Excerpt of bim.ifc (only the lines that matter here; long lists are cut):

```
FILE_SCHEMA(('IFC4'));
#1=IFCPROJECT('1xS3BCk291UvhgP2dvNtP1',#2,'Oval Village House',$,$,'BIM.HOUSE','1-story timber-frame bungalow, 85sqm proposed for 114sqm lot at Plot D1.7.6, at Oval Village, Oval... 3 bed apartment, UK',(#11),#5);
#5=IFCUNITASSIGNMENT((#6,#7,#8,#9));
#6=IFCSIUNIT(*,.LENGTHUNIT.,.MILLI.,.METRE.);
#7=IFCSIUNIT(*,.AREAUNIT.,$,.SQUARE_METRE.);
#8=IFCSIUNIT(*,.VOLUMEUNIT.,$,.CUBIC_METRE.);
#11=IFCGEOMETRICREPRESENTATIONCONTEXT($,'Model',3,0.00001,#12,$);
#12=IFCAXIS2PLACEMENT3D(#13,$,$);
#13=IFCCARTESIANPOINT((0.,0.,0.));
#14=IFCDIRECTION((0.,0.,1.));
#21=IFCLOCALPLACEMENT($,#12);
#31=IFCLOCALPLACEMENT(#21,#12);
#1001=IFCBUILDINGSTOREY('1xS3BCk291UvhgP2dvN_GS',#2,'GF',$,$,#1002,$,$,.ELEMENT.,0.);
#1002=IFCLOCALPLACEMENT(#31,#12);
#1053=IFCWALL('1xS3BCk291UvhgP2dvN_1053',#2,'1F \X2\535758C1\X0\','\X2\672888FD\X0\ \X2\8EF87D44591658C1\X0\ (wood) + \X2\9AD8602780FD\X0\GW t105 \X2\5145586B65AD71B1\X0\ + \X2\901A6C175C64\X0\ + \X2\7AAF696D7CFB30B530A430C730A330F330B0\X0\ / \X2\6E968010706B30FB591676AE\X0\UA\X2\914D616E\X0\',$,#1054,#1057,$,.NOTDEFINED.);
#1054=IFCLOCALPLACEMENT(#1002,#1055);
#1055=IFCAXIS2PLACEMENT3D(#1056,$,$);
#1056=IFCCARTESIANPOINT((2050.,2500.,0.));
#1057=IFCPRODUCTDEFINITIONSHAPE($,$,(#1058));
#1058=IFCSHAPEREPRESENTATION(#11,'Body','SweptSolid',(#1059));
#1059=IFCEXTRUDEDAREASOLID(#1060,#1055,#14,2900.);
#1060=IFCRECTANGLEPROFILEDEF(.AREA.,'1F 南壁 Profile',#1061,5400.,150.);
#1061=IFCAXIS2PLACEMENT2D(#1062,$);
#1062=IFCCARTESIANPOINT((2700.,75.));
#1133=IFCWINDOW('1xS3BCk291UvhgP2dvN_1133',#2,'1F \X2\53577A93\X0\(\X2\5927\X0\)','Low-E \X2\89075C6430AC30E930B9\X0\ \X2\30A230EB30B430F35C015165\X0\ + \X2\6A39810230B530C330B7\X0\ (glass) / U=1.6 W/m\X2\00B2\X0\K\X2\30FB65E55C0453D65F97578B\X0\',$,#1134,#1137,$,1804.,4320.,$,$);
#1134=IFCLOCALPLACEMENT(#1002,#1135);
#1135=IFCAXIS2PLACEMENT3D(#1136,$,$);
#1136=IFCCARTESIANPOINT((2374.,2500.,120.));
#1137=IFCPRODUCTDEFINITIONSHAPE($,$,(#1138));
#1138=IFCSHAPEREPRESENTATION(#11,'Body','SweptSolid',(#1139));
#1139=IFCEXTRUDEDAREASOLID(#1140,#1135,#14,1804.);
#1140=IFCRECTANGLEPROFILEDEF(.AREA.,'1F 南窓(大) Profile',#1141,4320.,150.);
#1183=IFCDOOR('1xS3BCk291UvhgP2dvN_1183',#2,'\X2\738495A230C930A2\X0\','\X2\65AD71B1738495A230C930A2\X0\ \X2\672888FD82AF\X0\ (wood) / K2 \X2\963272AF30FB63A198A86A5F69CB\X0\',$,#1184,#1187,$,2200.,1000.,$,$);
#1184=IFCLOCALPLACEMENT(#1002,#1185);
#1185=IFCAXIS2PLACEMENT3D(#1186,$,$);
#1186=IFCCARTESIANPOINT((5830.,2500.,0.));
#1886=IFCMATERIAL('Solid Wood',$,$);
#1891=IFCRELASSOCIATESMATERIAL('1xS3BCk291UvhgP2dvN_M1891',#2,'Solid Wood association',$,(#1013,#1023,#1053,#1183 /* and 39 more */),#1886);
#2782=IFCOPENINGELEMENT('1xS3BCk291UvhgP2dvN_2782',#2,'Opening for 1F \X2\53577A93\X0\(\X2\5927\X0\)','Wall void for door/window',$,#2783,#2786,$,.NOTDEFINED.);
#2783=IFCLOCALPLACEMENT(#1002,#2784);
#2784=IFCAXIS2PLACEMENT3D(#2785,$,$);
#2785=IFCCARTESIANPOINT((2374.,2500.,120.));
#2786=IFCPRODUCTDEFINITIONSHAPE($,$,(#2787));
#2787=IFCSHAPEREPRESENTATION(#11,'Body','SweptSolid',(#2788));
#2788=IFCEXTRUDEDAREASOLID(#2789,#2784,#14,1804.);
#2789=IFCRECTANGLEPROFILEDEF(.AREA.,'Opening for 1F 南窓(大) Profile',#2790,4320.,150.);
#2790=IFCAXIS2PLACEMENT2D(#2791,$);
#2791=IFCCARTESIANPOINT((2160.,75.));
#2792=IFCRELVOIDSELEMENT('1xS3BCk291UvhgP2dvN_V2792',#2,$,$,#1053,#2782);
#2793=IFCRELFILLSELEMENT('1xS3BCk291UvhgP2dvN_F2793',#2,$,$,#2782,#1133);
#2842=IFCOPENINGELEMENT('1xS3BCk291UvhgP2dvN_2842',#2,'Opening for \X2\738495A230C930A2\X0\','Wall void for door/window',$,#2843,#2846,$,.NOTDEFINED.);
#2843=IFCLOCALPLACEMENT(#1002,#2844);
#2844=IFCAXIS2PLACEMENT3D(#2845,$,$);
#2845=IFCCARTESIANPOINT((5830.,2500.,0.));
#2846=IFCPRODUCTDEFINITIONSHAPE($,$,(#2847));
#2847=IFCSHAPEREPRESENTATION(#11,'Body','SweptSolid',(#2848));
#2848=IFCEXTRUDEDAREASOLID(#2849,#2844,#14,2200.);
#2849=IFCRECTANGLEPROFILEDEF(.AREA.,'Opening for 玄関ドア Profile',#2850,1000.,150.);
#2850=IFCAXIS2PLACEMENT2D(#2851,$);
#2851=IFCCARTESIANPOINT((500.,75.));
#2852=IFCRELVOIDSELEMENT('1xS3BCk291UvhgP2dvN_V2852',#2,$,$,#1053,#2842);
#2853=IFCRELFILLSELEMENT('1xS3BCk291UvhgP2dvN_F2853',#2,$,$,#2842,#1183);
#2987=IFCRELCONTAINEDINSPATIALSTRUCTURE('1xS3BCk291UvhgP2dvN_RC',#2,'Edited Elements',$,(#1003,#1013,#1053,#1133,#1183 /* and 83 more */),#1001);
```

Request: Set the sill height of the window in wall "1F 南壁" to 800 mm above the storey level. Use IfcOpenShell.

```python
import numpy as np
import ifcopenshell
import ifcopenshell.api.geometry
import ifcopenshell.geom
import ifcopenshell.util.element
import ifcopenshell.util.placement
import ifcopenshell.util.shape
import ifcopenshell.util.unit

model = ifcopenshell.open("bim.ifc")
unit_scale = ifcopenshell.util.unit.calculate_unit_scale(model)

window = model.by_guid("1xS3BCk291UvhgP2dvN_1133")
opening = window.FillsVoids[0].RelatingOpeningElement
storey = ifcopenshell.util.element.get_container(window, ifc_class="IfcBuildingStorey")
level = ifcopenshell.util.placement.get_local_placement(storey.ObjectPlacement)[2, 3]

# The opening's origin need not be at the sill, so measure its lowest point.
shape = ifcopenshell.geom.create_shape(ifcopenshell.geom.settings(), opening)
bottom = ifcopenshell.util.shape.get_shape_bottom_elevation(shape, shape.geometry) / unit_scale
dz = level + 800.0 - bottom

shift = np.array([0.0, 0.0, dz])
# The window is not placed relative to its opening, so move both.
for product in (opening, window):
    matrix = ifcopenshell.util.placement.get_local_placement(product.ObjectPlacement)
    matrix[:3, 3] += shift
    ifcopenshell.api.geometry.edit_object_placement(model, product=product, matrix=matrix, is_si=False)

print(f"moved by {dz * unit_scale:+.3f} m")

model.write("bim-out.ifc")
```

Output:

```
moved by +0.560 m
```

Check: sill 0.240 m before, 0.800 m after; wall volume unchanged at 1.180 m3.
